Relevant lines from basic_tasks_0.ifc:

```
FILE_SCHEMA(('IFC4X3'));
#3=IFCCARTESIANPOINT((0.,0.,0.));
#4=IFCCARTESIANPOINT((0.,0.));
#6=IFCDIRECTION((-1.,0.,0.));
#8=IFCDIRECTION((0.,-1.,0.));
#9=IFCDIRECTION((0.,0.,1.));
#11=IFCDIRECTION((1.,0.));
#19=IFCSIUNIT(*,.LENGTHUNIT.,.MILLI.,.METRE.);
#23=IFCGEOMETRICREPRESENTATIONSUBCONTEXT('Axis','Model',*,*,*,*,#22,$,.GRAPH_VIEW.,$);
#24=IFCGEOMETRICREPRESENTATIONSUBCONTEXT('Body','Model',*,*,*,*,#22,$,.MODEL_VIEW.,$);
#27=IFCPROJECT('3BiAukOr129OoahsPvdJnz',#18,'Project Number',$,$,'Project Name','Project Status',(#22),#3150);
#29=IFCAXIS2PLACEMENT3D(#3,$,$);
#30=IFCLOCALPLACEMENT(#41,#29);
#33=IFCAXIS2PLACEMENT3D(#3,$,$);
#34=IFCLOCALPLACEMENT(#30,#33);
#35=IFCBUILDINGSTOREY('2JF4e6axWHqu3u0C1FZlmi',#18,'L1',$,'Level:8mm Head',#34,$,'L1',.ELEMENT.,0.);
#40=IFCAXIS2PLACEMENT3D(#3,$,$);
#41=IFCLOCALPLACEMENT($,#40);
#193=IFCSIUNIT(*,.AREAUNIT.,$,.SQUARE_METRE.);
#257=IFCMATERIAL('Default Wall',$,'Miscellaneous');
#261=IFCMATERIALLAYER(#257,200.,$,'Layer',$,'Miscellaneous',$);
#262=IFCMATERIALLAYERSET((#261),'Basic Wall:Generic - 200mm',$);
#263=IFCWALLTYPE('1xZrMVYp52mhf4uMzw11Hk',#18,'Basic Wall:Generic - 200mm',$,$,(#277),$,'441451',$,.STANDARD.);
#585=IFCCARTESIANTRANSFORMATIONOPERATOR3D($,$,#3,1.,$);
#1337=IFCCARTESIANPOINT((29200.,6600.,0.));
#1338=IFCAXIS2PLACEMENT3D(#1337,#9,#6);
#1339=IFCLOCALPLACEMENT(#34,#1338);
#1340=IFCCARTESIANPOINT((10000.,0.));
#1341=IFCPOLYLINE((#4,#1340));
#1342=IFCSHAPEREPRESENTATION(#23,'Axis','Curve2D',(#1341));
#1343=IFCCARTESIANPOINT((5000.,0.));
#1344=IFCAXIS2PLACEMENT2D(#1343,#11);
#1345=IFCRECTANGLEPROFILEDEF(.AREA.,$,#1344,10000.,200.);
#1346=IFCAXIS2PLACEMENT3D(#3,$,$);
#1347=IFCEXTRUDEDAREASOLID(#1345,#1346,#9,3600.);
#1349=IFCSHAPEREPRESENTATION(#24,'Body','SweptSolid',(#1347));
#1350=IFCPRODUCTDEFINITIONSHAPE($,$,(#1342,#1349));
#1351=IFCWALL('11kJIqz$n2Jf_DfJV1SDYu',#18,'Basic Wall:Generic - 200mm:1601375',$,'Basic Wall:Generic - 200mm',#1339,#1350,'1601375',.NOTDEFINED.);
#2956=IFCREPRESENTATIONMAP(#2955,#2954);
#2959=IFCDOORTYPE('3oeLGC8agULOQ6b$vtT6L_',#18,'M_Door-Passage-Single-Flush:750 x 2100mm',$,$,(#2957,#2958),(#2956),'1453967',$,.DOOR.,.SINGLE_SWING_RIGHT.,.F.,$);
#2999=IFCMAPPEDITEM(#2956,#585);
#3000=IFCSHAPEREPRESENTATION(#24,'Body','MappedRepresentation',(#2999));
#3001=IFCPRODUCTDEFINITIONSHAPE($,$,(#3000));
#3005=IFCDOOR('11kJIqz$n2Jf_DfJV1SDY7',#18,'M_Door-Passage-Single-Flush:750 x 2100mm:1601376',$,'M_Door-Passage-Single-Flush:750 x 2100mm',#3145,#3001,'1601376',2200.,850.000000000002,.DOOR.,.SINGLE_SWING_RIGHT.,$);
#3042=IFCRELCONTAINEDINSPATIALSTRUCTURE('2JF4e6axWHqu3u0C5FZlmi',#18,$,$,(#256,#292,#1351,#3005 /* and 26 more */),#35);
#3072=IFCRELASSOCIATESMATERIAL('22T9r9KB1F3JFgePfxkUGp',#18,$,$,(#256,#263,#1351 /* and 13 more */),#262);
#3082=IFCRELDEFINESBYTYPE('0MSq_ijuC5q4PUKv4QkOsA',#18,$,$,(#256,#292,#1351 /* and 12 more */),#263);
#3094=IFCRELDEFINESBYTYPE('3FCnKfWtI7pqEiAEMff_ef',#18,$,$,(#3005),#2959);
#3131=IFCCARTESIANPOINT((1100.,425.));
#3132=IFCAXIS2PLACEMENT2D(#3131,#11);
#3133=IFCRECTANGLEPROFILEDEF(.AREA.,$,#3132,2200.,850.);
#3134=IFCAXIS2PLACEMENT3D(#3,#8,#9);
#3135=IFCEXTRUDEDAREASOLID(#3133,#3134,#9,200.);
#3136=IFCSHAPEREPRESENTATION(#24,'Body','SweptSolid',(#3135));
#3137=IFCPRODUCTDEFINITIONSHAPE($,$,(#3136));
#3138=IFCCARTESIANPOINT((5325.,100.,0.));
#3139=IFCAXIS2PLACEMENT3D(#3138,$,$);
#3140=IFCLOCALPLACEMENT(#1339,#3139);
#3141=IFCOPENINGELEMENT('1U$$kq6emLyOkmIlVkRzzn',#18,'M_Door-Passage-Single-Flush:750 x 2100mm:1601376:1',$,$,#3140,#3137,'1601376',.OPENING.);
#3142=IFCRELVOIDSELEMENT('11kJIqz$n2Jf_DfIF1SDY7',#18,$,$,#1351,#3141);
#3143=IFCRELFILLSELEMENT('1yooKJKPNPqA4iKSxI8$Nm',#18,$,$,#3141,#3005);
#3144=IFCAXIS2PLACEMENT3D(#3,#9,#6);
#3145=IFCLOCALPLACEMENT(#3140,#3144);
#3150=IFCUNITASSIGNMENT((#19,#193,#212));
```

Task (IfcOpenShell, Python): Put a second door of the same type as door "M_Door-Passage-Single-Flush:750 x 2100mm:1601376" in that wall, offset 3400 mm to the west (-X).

```python
import ifcopenshell
import ifcopenshell.api.feature
import ifcopenshell.api.geometry
import ifcopenshell.api.root
import ifcopenshell.geom
import ifcopenshell.util.element
import ifcopenshell.util.placement
import ifcopenshell.util.shape
import ifcopenshell.util.unit

model = ifcopenshell.open("basic_tasks_0.ifc")
unit_scale = ifcopenshell.util.unit.calculate_unit_scale(model)
settings = ifcopenshell.geom.settings()


def volume(element):
    """Net volume in cubic metres, openings subtracted."""
    shape = ifcopenshell.geom.create_shape(settings, element)
    return ifcopenshell.util.shape.get_volume(shape.geometry)


def reuse_history(source, copy):
    """copy_class also copies each property set's owner history, people and application; keep the originals."""
    for rel in copy.IsDefinedBy:
        if rel.is_a("IfcRelDefinesByProperties") and (history := rel.RelatingPropertyDefinition.OwnerHistory):
            rel.RelatingPropertyDefinition.OwnerHistory = source.OwnerHistory
            ifcopenshell.util.element.remove_deep2(model, history)


door = model.by_guid("11kJIqz$n2Jf_DfJV1SDY7")
opening = door.FillsVoids[0].RelatingOpeningElement
wall = opening.VoidsElements[0].RelatingBuildingElement
before = volume(wall)
shift = ifcopenshell.util.placement.get_local_placement(wall.ObjectPlacement)[:3, 0] * 3.4 / unit_scale

# copy_class copies the void relationship, type, container and properties, but no geometry.
new_opening = ifcopenshell.api.root.copy_class(model, product=opening)
new_opening.Representation = ifcopenshell.util.element.copy_deep(
    model, opening.Representation, exclude=["IfcGeometricRepresentationContext", "IfcRepresentationMap"]
)
new_opening.Name = "M_Door-Passage-Single-Flush:750 x 2100mm"
new_opening.Tag = None
new_door = ifcopenshell.api.root.copy_class(model, product=door)
new_door.Representation = ifcopenshell.util.element.copy_deep(
    model, door.Representation, exclude=["IfcGeometricRepresentationContext", "IfcRepresentationMap"]
)
new_door.Name = "M_Door-Passage-Single-Flush:750 x 2100mm"
new_door.Tag = None
reuse_history(door, new_door)
ifcopenshell.api.feature.add_filling(model, opening=new_opening, element=new_door)

for old, new in ((opening, new_opening), (door, new_door)):
    matrix = ifcopenshell.util.placement.get_local_placement(old.ObjectPlacement)
    matrix[:3, 3] += shift
    ifcopenshell.api.geometry.edit_object_placement(model, product=new, matrix=matrix, is_si=False)

after = volume(wall)

print(f"wall volume {before:.3f} -> {after:.3f} m3")

model.write("basic_tasks_0_rev.ifc")
```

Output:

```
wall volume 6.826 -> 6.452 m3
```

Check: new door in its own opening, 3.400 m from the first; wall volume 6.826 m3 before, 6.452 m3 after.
